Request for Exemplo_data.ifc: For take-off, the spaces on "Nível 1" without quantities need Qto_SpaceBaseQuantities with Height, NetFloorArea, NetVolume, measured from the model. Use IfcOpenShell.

First a look at what the model holds.

```python
import ifcopenshell
import ifcopenshell.util.element
import ifcopenshell.util.unit

model = ifcopenshell.open("Exemplo_data.ifc")
print(model.schema)
for unit_type in ("LENGTHUNIT", "AREAUNIT", "VOLUMEUNIT"):
    print(unit_type, ifcopenshell.util.unit.calculate_unit_scale(model, unit_type))
storey = next(s for s in model.by_type("IfcBuildingStorey") if s.Name == "Nível 1")
spaces = [e for e in ifcopenshell.util.element.get_decomposition(storey) if e.is_a("IfcSpace")]
for e in sorted(spaces, key=lambda e: e.id()):
    print(e.id(), e.is_a(), e.Name, list(ifcopenshell.util.element.get_psets(e, qtos_only=True)), sep=" | ")
```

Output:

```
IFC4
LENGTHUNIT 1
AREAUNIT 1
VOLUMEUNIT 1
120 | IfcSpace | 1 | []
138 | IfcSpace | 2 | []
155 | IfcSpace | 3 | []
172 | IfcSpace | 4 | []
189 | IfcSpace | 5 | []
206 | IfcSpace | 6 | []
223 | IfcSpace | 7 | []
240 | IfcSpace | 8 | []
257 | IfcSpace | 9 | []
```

```python
import ifcopenshell
import ifcopenshell.api.pset
import ifcopenshell.geom
import ifcopenshell.util.element
import ifcopenshell.util.shape
import ifcopenshell.util.unit

model = ifcopenshell.open("Exemplo_data.ifc")
unit_scale = ifcopenshell.util.unit.calculate_unit_scale(model)
area_scale = ifcopenshell.util.unit.calculate_unit_scale(model, "AREAUNIT")
volume_scale = ifcopenshell.util.unit.calculate_unit_scale(model, "VOLUMEUNIT")
settings = ifcopenshell.geom.settings()

storey = next(s for s in model.by_type("IfcBuildingStorey") if s.Name == "Nível 1")
spaces = [e for e in ifcopenshell.util.element.get_decomposition(storey) if e.is_a("IfcSpace")]

for e in sorted(spaces, key=lambda e: e.id()):
    if ifcopenshell.util.element.get_psets(e, qtos_only=True, should_inherit=False):
        continue
    # Geometry comes back in metres, in the element's own axes.
    shape = ifcopenshell.geom.create_shape(settings, e)
    values = {
        "Height": ifcopenshell.util.shape.get_z(shape.geometry) / unit_scale,
        "NetFloorArea": ifcopenshell.util.shape.get_footprint_area(shape.geometry) / area_scale,
        "NetVolume": ifcopenshell.util.shape.get_volume(shape.geometry) / volume_scale,
    }
    qto = ifcopenshell.api.pset.add_qto(model, product=e, name="Qto_SpaceBaseQuantities")
    ifcopenshell.api.pset.edit_qto(model, qto=qto, properties=values)
    print(e.id(), {k: round(v, 3) for k, v in values.items()})

model.write("Exemplo_data_v2.ifc")
```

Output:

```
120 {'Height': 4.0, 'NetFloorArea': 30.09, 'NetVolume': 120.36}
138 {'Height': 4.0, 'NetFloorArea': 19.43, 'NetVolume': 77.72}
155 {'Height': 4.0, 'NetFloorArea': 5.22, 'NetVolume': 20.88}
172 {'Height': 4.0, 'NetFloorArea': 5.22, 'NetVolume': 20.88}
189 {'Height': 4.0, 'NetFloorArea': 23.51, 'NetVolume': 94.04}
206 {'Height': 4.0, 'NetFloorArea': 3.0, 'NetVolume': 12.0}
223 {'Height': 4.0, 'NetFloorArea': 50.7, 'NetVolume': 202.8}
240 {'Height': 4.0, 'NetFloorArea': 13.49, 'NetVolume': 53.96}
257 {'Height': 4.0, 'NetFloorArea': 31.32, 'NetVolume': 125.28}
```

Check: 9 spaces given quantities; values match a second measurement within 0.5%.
